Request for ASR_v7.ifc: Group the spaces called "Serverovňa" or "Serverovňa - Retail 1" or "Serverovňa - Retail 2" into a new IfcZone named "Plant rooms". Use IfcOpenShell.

First a look at what the model holds.

```python
import ifcopenshell

model = ifcopenshell.open("ASR_v7.ifc")
print(model.schema)
seen = {}
for space in model.by_type("IfcSpace"):
    seen[space.LongName] = seen.get(space.LongName, 0) + 1
for name, count in sorted(seen.items(), key=str):
    print(count, "x", name)
print("zones:", [z.Name for z in model.by_type("IfcZone")][:20])
```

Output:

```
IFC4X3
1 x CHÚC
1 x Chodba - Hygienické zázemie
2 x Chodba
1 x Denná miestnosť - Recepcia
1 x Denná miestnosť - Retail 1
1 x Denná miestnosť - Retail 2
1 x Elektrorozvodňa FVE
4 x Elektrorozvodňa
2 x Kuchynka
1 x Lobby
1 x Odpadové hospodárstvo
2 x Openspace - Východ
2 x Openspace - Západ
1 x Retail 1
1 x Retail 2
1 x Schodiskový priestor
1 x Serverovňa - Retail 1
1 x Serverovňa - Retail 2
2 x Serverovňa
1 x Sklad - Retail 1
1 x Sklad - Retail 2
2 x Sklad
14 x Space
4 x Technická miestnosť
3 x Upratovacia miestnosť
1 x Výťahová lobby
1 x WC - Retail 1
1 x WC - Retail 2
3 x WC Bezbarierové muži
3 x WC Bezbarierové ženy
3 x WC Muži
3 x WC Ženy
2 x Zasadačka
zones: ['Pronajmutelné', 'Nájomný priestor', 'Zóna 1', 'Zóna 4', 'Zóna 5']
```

```python
import ifcopenshell
import ifcopenshell.api.group
import ifcopenshell.api.root

model = ifcopenshell.open("ASR_v7.ifc")

names = {"Serverovňa", "Serverovňa - Retail 1", "Serverovňa - Retail 2"}
spaces = [s for s in model.by_type("IfcSpace") if s.LongName in names]

zone = ifcopenshell.api.root.create_entity(model, ifc_class="IfcZone", name="Plant rooms")
ifcopenshell.api.group.assign_group(model, products=spaces, group=zone)
print(len(spaces), "spaces in", zone.Name)

model.write("ASR_v7_updated.ifc")
```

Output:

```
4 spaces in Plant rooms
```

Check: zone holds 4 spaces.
